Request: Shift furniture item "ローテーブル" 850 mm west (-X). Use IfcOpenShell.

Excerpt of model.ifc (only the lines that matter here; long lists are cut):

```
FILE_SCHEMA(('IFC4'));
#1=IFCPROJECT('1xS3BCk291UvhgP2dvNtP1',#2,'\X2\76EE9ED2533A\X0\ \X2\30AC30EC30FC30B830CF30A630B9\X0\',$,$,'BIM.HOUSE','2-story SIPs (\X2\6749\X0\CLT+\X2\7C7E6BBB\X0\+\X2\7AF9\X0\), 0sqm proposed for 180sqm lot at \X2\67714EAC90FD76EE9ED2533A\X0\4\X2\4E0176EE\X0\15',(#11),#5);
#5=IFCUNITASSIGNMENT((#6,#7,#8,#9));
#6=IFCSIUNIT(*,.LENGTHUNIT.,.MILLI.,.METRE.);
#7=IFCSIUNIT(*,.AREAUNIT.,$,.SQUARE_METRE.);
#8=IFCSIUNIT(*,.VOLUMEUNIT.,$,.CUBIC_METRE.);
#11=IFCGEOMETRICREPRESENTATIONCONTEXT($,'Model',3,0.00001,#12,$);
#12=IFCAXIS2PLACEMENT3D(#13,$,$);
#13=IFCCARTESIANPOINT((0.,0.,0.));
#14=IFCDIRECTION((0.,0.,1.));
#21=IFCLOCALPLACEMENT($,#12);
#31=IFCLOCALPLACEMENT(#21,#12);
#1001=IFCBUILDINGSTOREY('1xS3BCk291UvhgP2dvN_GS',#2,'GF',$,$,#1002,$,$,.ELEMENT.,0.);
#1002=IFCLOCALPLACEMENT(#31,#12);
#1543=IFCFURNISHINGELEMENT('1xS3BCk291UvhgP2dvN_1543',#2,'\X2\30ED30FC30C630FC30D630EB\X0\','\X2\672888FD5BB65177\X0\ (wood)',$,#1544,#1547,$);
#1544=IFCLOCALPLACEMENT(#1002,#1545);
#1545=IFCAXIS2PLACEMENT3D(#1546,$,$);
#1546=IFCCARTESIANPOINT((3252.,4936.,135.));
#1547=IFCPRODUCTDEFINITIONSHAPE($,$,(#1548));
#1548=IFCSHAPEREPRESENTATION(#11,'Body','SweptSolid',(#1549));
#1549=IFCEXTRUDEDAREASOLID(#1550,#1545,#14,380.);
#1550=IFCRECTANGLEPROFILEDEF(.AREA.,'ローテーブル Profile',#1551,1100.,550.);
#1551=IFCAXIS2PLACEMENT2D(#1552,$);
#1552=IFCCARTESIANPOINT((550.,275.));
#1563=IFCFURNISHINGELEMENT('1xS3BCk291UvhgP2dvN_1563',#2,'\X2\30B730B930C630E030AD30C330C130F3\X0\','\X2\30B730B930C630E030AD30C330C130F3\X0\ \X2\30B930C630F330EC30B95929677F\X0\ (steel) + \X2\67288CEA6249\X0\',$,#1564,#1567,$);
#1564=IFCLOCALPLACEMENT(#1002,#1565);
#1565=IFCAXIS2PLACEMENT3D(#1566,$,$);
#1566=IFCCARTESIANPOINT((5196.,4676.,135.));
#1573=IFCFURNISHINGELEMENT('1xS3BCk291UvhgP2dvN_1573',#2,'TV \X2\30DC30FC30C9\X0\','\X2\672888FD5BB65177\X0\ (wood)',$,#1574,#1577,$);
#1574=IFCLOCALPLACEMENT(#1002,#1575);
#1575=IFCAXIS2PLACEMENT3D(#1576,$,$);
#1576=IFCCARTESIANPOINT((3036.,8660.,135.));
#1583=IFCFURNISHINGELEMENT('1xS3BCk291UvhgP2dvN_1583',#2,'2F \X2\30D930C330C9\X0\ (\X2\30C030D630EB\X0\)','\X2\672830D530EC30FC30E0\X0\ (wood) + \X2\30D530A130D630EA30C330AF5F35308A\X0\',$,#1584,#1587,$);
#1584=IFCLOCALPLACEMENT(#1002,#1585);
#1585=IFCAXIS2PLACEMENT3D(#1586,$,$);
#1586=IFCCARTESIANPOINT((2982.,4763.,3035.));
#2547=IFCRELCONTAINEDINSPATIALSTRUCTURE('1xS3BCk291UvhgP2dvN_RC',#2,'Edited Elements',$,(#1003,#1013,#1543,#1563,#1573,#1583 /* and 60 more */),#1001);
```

```python
import ifcopenshell
import ifcopenshell.api.geometry
import ifcopenshell.util.placement
import ifcopenshell.util.unit

model = ifcopenshell.open("model.ifc")
unit_scale = ifcopenshell.util.unit.calculate_unit_scale(model)

item = model.by_id(1543)
matrix = ifcopenshell.util.placement.get_local_placement(item.ObjectPlacement)
matrix[0, 3] -= 0.85 / unit_scale
ifcopenshell.api.geometry.edit_object_placement(model, product=item, matrix=matrix, is_si=False)

print(ifcopenshell.util.placement.get_local_placement(item.ObjectPlacement).round(3) + 0.0)

model.write("model_rev.ifc")
```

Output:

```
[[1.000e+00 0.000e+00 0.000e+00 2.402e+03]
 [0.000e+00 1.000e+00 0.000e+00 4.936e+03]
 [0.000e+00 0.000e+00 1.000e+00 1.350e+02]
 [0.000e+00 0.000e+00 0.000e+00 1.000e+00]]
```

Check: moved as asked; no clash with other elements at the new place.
